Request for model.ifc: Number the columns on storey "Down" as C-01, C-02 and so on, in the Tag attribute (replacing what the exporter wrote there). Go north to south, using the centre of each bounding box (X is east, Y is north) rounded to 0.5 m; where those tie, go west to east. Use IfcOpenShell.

First a look at what the model holds.

```python
import ifcopenshell
import ifcopenshell.util.element
import ifcopenshell.util.placement

model = ifcopenshell.open("model.ifc")
print(model.schema)
storey = next(s for s in model.by_type("IfcBuildingStorey") if s.Name == "Down")
columns = [e for e in ifcopenshell.util.element.get_decomposition(storey) if e.is_a("IfcColumn")]
for e in sorted(columns, key=lambda e: e.id()):
    origin = ifcopenshell.util.placement.get_local_placement(e.ObjectPlacement)[:3, 3]
    print(e.id(), e.Tag, e.Name, origin.round(2) + 0.0, sep=" | ")
```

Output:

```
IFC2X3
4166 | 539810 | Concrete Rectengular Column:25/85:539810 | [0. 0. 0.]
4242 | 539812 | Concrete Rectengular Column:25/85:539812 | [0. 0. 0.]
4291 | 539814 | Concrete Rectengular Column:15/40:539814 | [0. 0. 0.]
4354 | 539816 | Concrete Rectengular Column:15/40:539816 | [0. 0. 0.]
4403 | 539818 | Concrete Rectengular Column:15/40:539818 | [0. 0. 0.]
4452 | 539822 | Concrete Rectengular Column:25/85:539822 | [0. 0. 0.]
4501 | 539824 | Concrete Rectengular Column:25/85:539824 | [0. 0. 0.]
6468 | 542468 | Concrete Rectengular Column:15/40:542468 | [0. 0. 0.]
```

```python
import ifcopenshell
import ifcopenshell.geom
import ifcopenshell.util.element
import ifcopenshell.util.shape

model = ifcopenshell.open("model.ifc")
settings = ifcopenshell.geom.settings()
settings.set("use-world-coords", True)


def centre(element):
    shape = ifcopenshell.geom.create_shape(settings, element)
    return ifcopenshell.util.shape.get_bbox_centroid(shape.geometry)


storey = next(s for s in model.by_type("IfcBuildingStorey") if s.Name == "Down")
columns = [e for e in ifcopenshell.util.element.get_decomposition(storey) if e.is_a("IfcColumn")]

# Insertion points can sit at a corner or the storey origin, so sort by the geometry (in metres).
centres = {e: centre(e) for e in columns}
columns.sort(key=lambda e: (-round(centres[e][1] / 0.5), centres[e][0]))

for i, e in enumerate(columns, start=1):
    number = f"C-{i:02d}"
    e.Tag = number
    print(e.id(), number)

model.write("model_edited.ifc")
```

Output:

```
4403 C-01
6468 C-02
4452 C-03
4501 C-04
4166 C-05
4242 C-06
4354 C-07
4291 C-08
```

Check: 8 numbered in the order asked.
